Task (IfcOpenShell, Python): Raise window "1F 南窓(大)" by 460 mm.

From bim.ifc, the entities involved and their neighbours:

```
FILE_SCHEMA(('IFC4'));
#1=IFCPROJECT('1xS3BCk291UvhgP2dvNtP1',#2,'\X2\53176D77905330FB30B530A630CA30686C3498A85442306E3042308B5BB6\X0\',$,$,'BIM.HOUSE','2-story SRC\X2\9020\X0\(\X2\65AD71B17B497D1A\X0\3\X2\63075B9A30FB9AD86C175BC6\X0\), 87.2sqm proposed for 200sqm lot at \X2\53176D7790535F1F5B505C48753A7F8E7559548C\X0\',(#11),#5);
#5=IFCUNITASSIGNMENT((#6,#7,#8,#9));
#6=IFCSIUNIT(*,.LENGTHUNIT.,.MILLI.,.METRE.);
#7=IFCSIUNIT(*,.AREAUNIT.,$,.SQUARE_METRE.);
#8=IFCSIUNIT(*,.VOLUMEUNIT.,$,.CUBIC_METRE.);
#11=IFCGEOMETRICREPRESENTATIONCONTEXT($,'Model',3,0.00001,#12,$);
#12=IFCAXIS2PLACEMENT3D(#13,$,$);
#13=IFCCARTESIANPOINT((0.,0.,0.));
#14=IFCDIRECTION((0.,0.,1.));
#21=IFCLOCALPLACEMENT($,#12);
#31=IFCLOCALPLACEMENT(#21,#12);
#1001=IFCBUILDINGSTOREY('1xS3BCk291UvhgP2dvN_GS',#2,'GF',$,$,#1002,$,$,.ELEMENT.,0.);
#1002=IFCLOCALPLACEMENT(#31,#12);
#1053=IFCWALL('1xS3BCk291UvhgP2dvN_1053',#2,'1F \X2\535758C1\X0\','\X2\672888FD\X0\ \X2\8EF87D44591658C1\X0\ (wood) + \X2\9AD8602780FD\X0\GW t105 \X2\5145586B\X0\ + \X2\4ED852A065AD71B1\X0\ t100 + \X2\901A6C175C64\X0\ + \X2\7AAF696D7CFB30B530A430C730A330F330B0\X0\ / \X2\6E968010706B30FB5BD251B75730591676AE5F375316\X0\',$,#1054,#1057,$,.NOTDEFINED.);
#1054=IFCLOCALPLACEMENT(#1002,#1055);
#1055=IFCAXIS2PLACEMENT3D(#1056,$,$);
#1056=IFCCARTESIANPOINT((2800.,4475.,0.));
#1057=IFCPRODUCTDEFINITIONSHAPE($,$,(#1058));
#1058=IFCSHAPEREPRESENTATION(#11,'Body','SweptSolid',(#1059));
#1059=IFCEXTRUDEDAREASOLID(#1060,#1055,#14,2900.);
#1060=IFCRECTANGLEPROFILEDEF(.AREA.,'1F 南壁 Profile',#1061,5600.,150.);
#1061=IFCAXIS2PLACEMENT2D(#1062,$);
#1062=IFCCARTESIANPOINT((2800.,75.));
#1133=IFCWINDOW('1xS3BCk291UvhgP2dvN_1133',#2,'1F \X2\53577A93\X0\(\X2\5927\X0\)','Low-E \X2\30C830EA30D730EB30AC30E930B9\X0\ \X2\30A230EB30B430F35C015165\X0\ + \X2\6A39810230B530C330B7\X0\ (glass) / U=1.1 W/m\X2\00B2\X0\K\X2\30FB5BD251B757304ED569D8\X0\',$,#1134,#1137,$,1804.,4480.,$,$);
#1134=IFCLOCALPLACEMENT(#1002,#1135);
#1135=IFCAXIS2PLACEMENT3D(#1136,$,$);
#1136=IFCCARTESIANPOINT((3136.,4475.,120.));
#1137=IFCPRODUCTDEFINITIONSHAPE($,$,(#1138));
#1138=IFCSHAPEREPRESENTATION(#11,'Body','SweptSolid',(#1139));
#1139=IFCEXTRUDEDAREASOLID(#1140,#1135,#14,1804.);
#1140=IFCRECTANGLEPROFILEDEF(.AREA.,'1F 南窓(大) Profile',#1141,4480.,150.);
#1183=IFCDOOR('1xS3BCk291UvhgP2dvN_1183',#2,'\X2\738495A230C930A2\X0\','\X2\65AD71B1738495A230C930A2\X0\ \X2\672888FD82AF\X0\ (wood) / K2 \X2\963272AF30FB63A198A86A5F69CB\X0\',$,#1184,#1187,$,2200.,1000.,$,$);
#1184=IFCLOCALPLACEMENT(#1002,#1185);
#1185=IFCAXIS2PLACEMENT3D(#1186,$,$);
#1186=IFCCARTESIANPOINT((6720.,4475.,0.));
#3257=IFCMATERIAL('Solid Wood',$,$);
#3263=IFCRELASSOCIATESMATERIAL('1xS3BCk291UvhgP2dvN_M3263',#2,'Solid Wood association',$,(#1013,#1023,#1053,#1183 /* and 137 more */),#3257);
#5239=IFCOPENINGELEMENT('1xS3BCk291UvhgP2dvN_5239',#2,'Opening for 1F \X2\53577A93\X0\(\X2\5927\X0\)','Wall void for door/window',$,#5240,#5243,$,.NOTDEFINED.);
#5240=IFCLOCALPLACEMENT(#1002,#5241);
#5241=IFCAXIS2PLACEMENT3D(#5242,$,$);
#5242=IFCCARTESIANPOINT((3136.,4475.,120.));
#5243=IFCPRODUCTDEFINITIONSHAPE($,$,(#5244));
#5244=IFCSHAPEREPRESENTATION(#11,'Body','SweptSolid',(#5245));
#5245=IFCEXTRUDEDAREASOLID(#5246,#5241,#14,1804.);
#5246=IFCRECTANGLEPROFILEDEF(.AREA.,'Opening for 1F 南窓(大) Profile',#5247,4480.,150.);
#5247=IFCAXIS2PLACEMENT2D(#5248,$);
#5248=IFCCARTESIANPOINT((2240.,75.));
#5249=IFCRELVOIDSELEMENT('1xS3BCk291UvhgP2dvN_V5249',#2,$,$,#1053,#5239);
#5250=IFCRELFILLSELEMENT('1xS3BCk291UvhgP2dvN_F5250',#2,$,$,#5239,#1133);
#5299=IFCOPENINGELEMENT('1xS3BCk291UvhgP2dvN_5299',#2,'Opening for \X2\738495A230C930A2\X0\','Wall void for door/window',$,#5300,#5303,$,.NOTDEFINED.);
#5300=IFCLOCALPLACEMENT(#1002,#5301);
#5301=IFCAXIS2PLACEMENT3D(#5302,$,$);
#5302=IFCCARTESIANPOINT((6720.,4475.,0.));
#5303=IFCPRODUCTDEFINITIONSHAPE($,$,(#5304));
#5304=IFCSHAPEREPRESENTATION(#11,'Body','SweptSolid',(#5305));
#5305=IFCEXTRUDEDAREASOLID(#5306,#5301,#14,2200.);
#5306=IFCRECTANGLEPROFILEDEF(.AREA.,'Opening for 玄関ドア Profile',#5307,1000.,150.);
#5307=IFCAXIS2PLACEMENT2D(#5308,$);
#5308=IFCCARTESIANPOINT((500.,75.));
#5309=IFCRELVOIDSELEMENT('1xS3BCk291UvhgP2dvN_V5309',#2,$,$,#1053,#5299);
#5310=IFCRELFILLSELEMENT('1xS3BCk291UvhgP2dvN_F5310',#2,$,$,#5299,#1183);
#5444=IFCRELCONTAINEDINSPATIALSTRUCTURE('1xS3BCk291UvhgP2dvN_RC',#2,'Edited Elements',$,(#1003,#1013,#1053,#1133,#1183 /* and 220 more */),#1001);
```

```python
import numpy as np
import ifcopenshell
import ifcopenshell.api.geometry
import ifcopenshell.util.placement
import ifcopenshell.util.unit

model = ifcopenshell.open("bim.ifc")
unit_scale = ifcopenshell.util.unit.calculate_unit_scale(model)

window = model.by_id(1133)
opening = window.FillsVoids[0].RelatingOpeningElement
dz = 0.46 / unit_scale

shift = np.array([0.0, 0.0, dz])
# The window is not placed relative to its opening, so move both.
for product in (opening, window):
    matrix = ifcopenshell.util.placement.get_local_placement(product.ObjectPlacement)
    matrix[:3, 3] += shift
    ifcopenshell.api.geometry.edit_object_placement(model, product=product, matrix=matrix, is_si=False)

print(f"moved by {dz * unit_scale:+.3f} m")

model.write("bim_rev.ifc")
```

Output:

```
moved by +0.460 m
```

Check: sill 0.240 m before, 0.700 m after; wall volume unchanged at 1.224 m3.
